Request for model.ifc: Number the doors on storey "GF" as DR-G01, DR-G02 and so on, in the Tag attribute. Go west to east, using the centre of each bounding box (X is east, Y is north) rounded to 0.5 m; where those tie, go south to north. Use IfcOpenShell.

First a look at what the model holds.

```python
import ifcopenshell
import ifcopenshell.util.element
import ifcopenshell.util.placement

model = ifcopenshell.open("model.ifc")
print(model.schema)
storey = next(s for s in model.by_type("IfcBuildingStorey") if s.Name == "GF")
doors = [e for e in ifcopenshell.util.element.get_decomposition(storey) if e.is_a("IfcDoor")]
for e in sorted(doors, key=lambda e: e.id()):
    origin = ifcopenshell.util.placement.get_local_placement(e.ObjectPlacement)[:3, 3]
    print(e.id(), e.Tag, e.Name, origin.round(2) + 0.0, sep=" | ")
```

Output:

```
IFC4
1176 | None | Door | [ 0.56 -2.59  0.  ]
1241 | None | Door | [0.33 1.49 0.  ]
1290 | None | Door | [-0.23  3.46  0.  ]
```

```python
import ifcopenshell
import ifcopenshell.geom
import ifcopenshell.util.element
import ifcopenshell.util.shape

model = ifcopenshell.open("model.ifc")
settings = ifcopenshell.geom.settings()
settings.set("use-world-coords", True)


def centre(element):
    shape = ifcopenshell.geom.create_shape(settings, element)
    return ifcopenshell.util.shape.get_bbox_centroid(shape.geometry)


storey = next(s for s in model.by_type("IfcBuildingStorey") if s.Name == "GF")
doors = [e for e in ifcopenshell.util.element.get_decomposition(storey) if e.is_a("IfcDoor")]

# Insertion points can sit at a corner or the storey origin, so sort by the geometry (in metres).
centres = {e: centre(e) for e in doors}
doors.sort(key=lambda e: (round(centres[e][0] / 0.5), centres[e][1]))

for i, e in enumerate(doors, start=1):
    number = f"DR-G{i:02d}"
    e.Tag = number
    print(e.id(), number)

model.write("model_rev.ifc")
```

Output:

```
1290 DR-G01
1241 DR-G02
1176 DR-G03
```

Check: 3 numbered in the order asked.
